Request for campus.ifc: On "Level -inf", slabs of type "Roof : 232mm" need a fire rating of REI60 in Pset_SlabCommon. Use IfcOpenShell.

First a look at what the model holds.

```python
import ifcopenshell
import ifcopenshell.util.element

model = ifcopenshell.open("campus.ifc")
print(model.schema)
storey = next(s for s in model.by_type("IfcBuildingStorey") if s.Name == "Level -inf")
slabs = [e for e in ifcopenshell.util.element.get_decomposition(storey) if e.is_a("IfcSlab")]
seen = {}
for e in slabs:
    element_type = ifcopenshell.util.element.get_type(e)
    key = (element_type.Name if element_type != e and element_type else None, ifcopenshell.util.element.get_pset(e, "Pset_SlabCommon", "FireRating"))
    seen[key] = seen.get(key, 0) + 1
for (name, value), count in sorted(seen.items(), key=str):
    print(count, "x", name, "|", value)
```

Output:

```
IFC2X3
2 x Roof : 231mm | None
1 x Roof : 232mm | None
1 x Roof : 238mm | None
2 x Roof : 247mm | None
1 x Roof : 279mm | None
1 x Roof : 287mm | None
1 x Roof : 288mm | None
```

```python
import ifcopenshell
import ifcopenshell.api.pset
import ifcopenshell.util.element

model = ifcopenshell.open("campus.ifc")

storey = next(s for s in model.by_type("IfcBuildingStorey") if s.Name == "Level -inf")
slabs = [e for e in ifcopenshell.util.element.get_decomposition(storey) if e.is_a("IfcSlab")]

count = 0
for e in slabs:
    element_type = ifcopenshell.util.element.get_type(e)
    if element_type in (None, e) or element_type.Name != "Roof : 232mm":
        continue
    # add_pset returns the element's existing set when there is one.
    pset = ifcopenshell.api.pset.add_pset(model, product=e, name="Pset_SlabCommon")
    ifcopenshell.api.pset.edit_pset(model, pset=pset, properties={"FireRating": "REI60"})
    count += 1

print(count, "slabs updated")

model.write("campus_edited.ifc")
```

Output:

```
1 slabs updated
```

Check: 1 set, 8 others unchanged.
